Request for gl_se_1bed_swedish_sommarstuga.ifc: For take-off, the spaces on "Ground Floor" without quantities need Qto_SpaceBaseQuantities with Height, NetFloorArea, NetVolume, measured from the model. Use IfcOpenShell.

First a look at what the model holds.

```python
import ifcopenshell
import ifcopenshell.util.element
import ifcopenshell.util.unit

model = ifcopenshell.open("gl_se_1bed_swedish_sommarstuga.ifc")
print(model.schema)
for unit_type in ("LENGTHUNIT", "AREAUNIT", "VOLUMEUNIT"):
    print(unit_type, ifcopenshell.util.unit.calculate_unit_scale(model, unit_type))
storey = next(s for s in model.by_type("IfcBuildingStorey") if s.Name == "Ground Floor")
spaces = [e for e in ifcopenshell.util.element.get_decomposition(storey) if e.is_a("IfcSpace")]
for e in sorted(spaces, key=lambda e: e.id()):
    print(e.id(), e.is_a(), e.Name, list(ifcopenshell.util.element.get_psets(e, qtos_only=True)), sep=" | ")
```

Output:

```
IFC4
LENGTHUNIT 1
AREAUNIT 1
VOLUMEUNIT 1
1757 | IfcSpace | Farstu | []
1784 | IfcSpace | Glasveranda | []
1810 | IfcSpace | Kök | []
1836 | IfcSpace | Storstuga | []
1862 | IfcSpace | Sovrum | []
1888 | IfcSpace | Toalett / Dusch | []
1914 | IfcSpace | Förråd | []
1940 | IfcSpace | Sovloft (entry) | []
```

```python
import ifcopenshell
import ifcopenshell.api.pset
import ifcopenshell.geom
import ifcopenshell.util.element
import ifcopenshell.util.shape
import ifcopenshell.util.unit

model = ifcopenshell.open("gl_se_1bed_swedish_sommarstuga.ifc")
unit_scale = ifcopenshell.util.unit.calculate_unit_scale(model)
area_scale = ifcopenshell.util.unit.calculate_unit_scale(model, "AREAUNIT")
volume_scale = ifcopenshell.util.unit.calculate_unit_scale(model, "VOLUMEUNIT")
settings = ifcopenshell.geom.settings()

storey = next(s for s in model.by_type("IfcBuildingStorey") if s.Name == "Ground Floor")
spaces = [e for e in ifcopenshell.util.element.get_decomposition(storey) if e.is_a("IfcSpace")]

for e in sorted(spaces, key=lambda e: e.id()):
    if ifcopenshell.util.element.get_psets(e, qtos_only=True, should_inherit=False):
        continue
    # Geometry comes back in metres, in the element's own axes.
    shape = ifcopenshell.geom.create_shape(settings, e)
    values = {
        "Height": ifcopenshell.util.shape.get_z(shape.geometry) / unit_scale,
        "NetFloorArea": ifcopenshell.util.shape.get_footprint_area(shape.geometry) / area_scale,
        "NetVolume": ifcopenshell.util.shape.get_volume(shape.geometry) / volume_scale,
    }
    qto = ifcopenshell.api.pset.add_qto(model, product=e, name="Qto_SpaceBaseQuantities")
    ifcopenshell.api.pset.edit_qto(model, qto=qto, properties=values)
    print(e.id(), {k: round(v, 3) for k, v in values.items()})

model.write("gl_se_1bed_swedish_sommarstuga_rev.ifc")
```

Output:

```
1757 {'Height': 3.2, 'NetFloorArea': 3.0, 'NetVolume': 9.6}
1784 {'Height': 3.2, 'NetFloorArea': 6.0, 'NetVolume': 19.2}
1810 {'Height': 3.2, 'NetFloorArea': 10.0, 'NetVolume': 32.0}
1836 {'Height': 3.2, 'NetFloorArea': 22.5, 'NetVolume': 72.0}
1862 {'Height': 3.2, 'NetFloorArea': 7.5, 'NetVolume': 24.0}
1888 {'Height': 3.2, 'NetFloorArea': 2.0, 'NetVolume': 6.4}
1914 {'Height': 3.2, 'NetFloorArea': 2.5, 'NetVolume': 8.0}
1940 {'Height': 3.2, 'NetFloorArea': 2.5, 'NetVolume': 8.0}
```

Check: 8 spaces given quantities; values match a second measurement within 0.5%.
